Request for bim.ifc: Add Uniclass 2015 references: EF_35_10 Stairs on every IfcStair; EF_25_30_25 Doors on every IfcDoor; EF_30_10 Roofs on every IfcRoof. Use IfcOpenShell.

First a look at what the model holds.

```python
import ifcopenshell

model = ifcopenshell.open("bim.ifc")
print(model.schema)
print("classifications:", [c.Name for c in model.by_type("IfcClassification")])
for ifc_class in ("IfcDoor", "IfcRoof", "IfcStair", "IfcWall", "IfcWindow"):
    print(ifc_class, len(model.by_type(ifc_class)))
```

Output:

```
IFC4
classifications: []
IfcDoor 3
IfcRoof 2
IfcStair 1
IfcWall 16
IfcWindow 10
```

```python
import ifcopenshell
import ifcopenshell.api.classification

model = ifcopenshell.open("bim.ifc")

system = ifcopenshell.api.classification.add_classification(model, classification="Uniclass 2015")

codes = {
    "IfcStair": ("EF_35_10", "Stairs"),
    "IfcDoor": ("EF_25_30_25", "Doors"),
    "IfcRoof": ("EF_30_10", "Roofs"),
}
for ifc_class, (code, name) in codes.items():
    products = model.by_type(ifc_class)
    ifcopenshell.api.classification.add_reference(
        model, products=products, classification=system, identification=code, name=name
    )
    print(code, len(products))

model.write("bim_rev.ifc")
```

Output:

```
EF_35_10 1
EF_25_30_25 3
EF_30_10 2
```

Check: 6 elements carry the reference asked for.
